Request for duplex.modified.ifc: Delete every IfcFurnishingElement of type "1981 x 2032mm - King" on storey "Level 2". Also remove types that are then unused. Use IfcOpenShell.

First a look at what the model holds.

```python
import ifcopenshell
import ifcopenshell.util.element

model = ifcopenshell.open("duplex.modified.ifc")
print(model.schema)
storey = next(s for s in model.by_type("IfcBuildingStorey") if s.Name == "Level 2")
furniture = [e for e in ifcopenshell.util.element.get_decomposition(storey) if e.is_a("IfcFurnishingElement")]
seen = {}
for e in furniture:
    element_type = ifcopenshell.util.element.get_type(e)
    name = element_type.Name if element_type not in (None, e) else None
    seen[name] = seen.get(name, 0) + 1
for name, count in sorted(seen.items(), key=str):
    print(count, "x", name)
```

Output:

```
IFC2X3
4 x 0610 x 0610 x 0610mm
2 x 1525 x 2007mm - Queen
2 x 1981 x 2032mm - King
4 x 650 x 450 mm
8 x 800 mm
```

```python
import ifcopenshell
import ifcopenshell.api.root
import ifcopenshell.util.element

model = ifcopenshell.open("duplex.modified.ifc")

storey = next(s for s in model.by_type("IfcBuildingStorey") if s.Name == "Level 2")
furniture = [e for e in ifcopenshell.util.element.get_decomposition(storey) if e.is_a("IfcFurnishingElement")]
targets = [e for e in furniture if (t := ifcopenshell.util.element.get_type(e)) not in (None, e) and t.Name == "1981 x 2032mm - King"]
types = {ifcopenshell.util.element.get_type(e) for e in targets} - {None, *targets}

for e in targets:
    ifcopenshell.api.root.remove_product(model, product=e)
print(len(targets), "removed")

unused = [t for t in types if not ifcopenshell.util.element.get_types(t)]
for t in unused:
    ifcopenshell.api.root.remove_product(model, product=t)
print(len(unused), "unused types removed")

model.write("duplex.modified_updated.ifc")
```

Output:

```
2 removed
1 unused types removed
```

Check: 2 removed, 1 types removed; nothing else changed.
